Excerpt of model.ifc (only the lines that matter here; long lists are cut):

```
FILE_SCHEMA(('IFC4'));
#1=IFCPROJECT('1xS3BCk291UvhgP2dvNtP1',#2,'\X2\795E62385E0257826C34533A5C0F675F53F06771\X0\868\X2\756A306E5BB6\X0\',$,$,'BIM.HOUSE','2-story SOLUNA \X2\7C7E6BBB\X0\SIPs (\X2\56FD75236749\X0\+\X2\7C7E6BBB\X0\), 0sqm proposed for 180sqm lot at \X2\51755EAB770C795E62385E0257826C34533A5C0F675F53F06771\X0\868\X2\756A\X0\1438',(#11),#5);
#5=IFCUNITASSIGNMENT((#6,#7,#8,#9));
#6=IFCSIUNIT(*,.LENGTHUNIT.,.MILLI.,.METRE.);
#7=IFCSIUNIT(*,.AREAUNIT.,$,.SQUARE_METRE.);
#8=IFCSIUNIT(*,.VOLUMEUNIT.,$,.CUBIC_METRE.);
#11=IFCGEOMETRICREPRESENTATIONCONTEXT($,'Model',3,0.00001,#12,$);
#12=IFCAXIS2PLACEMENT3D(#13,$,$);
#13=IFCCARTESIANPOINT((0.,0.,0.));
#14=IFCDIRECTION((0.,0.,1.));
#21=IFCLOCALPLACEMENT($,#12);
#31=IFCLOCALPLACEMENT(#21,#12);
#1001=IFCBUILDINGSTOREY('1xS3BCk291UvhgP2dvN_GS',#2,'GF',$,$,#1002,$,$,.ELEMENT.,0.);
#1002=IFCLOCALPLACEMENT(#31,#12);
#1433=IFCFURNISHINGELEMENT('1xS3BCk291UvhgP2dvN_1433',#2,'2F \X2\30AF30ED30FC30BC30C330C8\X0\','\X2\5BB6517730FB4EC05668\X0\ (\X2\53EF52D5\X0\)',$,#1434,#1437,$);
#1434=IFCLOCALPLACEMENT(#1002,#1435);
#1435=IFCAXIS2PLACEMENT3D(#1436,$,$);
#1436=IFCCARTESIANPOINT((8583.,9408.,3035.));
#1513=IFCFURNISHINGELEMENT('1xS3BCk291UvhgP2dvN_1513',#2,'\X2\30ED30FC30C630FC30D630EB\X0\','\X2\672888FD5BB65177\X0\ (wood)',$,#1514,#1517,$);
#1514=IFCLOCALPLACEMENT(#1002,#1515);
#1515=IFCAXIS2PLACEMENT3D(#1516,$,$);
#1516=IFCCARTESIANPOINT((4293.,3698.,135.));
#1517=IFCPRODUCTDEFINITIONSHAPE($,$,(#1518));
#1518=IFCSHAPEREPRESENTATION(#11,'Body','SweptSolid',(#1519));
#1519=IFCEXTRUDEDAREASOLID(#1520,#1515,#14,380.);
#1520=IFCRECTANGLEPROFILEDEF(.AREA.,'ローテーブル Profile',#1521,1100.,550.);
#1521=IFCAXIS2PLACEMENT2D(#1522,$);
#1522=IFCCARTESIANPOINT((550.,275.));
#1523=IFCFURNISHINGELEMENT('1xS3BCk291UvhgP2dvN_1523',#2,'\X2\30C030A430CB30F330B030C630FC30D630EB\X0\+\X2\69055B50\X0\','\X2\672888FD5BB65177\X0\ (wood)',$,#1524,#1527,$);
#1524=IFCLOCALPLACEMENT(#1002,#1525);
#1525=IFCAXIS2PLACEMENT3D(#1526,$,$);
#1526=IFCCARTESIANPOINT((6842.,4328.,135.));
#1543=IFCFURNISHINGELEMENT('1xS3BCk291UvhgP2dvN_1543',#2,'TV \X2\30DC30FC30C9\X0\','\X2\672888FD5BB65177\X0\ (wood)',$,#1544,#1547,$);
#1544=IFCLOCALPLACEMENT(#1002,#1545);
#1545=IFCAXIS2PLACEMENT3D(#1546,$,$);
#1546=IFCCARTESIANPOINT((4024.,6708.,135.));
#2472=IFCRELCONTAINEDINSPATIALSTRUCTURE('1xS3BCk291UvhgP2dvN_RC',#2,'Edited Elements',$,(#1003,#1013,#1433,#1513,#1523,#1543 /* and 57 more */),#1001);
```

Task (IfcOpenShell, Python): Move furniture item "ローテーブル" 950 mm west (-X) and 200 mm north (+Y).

```python
import ifcopenshell
import ifcopenshell.api.geometry
import ifcopenshell.util.placement
import ifcopenshell.util.unit

model = ifcopenshell.open("model.ifc")
unit_scale = ifcopenshell.util.unit.calculate_unit_scale(model)

item = model.by_guid("1xS3BCk291UvhgP2dvN_1513")
matrix = ifcopenshell.util.placement.get_local_placement(item.ObjectPlacement)
matrix[0, 3] -= 0.95 / unit_scale
matrix[1, 3] += 0.2 / unit_scale
ifcopenshell.api.geometry.edit_object_placement(model, product=item, matrix=matrix, is_si=False)

print(ifcopenshell.util.placement.get_local_placement(item.ObjectPlacement).round(3) + 0.0)

model.write("model_edited.ifc")
```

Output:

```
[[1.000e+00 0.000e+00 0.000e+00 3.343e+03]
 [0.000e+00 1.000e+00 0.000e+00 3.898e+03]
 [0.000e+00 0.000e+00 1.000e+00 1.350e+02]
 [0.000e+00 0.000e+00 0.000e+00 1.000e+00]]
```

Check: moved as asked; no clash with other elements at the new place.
